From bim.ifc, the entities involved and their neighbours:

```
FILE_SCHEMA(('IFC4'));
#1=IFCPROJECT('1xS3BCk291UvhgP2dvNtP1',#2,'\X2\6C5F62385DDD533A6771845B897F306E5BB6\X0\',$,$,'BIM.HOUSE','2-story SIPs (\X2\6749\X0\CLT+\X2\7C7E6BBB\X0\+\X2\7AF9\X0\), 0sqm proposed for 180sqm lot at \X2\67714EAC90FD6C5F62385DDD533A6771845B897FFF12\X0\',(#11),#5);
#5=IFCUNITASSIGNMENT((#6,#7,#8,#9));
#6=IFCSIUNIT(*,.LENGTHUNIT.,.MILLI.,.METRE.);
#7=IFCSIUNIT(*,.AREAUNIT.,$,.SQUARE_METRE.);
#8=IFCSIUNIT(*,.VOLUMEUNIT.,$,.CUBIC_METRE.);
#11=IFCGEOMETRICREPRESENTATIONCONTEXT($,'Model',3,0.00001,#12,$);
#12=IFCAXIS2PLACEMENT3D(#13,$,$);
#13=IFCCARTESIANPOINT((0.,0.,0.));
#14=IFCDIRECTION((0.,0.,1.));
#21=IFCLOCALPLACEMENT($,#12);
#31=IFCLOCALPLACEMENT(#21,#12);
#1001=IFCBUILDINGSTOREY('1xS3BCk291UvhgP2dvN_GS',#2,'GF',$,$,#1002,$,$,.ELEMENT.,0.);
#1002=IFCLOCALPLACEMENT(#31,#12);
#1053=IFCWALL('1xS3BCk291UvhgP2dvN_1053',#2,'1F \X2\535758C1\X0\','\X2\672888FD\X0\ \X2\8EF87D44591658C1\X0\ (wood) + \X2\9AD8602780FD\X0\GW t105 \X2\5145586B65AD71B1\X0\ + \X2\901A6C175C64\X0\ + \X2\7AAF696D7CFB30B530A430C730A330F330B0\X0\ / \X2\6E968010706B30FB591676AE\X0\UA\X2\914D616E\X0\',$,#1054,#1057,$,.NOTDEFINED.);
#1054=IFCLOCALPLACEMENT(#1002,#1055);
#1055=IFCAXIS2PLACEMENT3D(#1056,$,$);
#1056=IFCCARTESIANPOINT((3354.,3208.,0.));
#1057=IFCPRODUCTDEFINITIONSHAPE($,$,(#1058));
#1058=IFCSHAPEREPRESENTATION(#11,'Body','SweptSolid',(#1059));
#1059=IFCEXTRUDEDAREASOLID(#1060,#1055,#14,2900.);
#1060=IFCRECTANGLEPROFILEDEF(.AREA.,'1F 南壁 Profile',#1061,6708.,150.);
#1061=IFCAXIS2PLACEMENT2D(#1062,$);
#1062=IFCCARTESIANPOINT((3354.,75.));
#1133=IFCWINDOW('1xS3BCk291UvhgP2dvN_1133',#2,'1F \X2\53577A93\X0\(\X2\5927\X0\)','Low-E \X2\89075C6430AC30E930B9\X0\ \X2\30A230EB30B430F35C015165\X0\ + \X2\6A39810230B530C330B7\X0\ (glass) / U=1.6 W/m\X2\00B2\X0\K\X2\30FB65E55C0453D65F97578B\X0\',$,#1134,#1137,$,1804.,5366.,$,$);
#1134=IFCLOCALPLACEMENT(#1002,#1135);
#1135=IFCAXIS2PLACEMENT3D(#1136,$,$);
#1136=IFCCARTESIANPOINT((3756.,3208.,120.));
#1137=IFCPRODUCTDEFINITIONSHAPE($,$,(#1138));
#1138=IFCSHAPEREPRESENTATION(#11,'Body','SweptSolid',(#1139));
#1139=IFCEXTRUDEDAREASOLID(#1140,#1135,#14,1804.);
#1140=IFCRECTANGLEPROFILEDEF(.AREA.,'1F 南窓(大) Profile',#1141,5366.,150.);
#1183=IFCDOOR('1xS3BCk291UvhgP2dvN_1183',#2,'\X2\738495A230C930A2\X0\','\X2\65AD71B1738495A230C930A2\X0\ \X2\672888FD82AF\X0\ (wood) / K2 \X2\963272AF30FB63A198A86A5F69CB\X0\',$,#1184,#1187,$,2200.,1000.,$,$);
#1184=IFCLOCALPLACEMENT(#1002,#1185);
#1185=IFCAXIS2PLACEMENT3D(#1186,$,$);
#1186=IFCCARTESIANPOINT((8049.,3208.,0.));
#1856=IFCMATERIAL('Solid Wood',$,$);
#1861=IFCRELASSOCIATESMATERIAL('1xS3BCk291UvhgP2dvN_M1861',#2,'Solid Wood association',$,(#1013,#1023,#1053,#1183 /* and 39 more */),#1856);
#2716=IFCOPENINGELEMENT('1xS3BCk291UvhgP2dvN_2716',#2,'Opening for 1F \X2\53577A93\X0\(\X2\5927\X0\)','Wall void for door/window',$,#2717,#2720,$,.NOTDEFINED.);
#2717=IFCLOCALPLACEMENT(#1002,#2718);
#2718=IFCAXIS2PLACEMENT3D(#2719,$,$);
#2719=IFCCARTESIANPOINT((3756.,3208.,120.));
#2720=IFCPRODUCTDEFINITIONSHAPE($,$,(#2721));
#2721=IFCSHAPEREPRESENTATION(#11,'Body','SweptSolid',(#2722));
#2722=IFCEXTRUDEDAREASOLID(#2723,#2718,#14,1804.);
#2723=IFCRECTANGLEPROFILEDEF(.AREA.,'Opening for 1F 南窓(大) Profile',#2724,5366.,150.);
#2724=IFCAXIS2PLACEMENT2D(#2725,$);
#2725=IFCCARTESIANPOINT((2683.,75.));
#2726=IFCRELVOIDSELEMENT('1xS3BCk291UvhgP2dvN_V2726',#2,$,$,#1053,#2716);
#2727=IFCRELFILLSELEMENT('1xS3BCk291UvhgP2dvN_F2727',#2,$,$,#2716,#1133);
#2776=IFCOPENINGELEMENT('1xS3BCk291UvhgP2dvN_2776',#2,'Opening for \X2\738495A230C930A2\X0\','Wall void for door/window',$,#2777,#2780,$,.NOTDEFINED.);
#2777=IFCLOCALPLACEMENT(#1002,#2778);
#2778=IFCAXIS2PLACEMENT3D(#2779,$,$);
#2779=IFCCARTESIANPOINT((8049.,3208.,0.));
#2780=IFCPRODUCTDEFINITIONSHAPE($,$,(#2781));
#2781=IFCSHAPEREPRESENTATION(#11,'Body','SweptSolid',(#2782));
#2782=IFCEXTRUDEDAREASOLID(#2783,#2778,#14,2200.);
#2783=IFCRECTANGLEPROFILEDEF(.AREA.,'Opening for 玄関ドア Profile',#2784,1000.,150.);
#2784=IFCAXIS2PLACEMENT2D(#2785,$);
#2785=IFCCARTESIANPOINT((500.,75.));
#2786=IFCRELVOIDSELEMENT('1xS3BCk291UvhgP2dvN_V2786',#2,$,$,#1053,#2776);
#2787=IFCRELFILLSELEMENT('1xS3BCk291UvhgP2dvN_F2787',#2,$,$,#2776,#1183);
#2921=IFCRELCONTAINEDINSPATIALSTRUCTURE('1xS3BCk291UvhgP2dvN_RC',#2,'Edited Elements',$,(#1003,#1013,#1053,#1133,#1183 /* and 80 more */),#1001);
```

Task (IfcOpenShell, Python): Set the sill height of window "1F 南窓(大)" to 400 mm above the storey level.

```python
import numpy as np
import ifcopenshell
import ifcopenshell.api.geometry
import ifcopenshell.geom
import ifcopenshell.util.element
import ifcopenshell.util.placement
import ifcopenshell.util.shape
import ifcopenshell.util.unit

model = ifcopenshell.open("bim.ifc")
unit_scale = ifcopenshell.util.unit.calculate_unit_scale(model)

window = model.by_guid("1xS3BCk291UvhgP2dvN_1133")
opening = window.FillsVoids[0].RelatingOpeningElement
storey = ifcopenshell.util.element.get_container(window, ifc_class="IfcBuildingStorey")
level = ifcopenshell.util.placement.get_local_placement(storey.ObjectPlacement)[2, 3]

# The opening's origin need not be at the sill, so measure its lowest point.
shape = ifcopenshell.geom.create_shape(ifcopenshell.geom.settings(), opening)
bottom = ifcopenshell.util.shape.get_shape_bottom_elevation(shape, shape.geometry) / unit_scale
dz = level + 0.4 / unit_scale - bottom

shift = np.array([0.0, 0.0, dz])
# The window is not placed relative to its opening, so move both.
for product in (opening, window):
    matrix = ifcopenshell.util.placement.get_local_placement(product.ObjectPlacement)
    matrix[:3, 3] += shift
    ifcopenshell.api.geometry.edit_object_placement(model, product=product, matrix=matrix, is_si=False)

print(f"moved by {dz * unit_scale:+.3f} m")

model.write("bim-out.ifc")
```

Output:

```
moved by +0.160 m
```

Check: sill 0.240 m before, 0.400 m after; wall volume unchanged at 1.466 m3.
